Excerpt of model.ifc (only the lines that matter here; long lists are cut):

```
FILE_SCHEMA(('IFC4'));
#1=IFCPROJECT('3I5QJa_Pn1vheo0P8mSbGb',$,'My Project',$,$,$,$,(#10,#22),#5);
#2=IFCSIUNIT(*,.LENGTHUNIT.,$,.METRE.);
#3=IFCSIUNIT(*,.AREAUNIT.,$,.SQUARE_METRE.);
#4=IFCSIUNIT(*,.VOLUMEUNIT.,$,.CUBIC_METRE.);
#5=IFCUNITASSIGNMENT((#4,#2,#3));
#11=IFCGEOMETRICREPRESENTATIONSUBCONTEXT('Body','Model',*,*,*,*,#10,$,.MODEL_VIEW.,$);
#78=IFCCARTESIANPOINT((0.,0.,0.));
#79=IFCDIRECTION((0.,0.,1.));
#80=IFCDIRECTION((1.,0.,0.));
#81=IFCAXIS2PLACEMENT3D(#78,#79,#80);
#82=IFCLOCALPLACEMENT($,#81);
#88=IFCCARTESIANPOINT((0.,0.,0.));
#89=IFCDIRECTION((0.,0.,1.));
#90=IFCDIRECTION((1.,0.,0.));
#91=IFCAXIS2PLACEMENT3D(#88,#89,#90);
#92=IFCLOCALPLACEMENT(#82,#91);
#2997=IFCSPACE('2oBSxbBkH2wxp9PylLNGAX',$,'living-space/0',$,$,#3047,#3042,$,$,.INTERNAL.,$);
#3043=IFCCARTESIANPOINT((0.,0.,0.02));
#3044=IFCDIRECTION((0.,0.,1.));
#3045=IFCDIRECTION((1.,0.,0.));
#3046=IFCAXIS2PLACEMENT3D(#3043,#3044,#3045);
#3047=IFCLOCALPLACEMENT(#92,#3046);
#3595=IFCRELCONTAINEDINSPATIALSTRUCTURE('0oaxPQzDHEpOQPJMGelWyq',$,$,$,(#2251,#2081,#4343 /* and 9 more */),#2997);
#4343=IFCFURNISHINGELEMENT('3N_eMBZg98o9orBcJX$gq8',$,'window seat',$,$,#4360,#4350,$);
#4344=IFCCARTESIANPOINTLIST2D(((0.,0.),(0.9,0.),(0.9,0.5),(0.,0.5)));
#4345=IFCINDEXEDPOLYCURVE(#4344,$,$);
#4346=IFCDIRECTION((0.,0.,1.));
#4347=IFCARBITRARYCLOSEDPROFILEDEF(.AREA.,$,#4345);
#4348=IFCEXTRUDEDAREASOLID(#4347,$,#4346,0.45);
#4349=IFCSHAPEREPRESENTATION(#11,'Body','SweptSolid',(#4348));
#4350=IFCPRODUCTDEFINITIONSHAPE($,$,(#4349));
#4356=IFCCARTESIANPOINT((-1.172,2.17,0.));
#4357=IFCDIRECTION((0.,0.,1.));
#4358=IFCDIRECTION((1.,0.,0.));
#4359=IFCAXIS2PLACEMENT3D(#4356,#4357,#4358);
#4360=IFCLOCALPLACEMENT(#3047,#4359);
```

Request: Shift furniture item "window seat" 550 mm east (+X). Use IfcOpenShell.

```python
import ifcopenshell
import ifcopenshell.api.geometry
import ifcopenshell.util.placement
import ifcopenshell.util.unit

model = ifcopenshell.open("model.ifc")
unit_scale = ifcopenshell.util.unit.calculate_unit_scale(model)

item = model.by_guid("3N_eMBZg98o9orBcJX$gq8")
matrix = ifcopenshell.util.placement.get_local_placement(item.ObjectPlacement)
matrix[0, 3] += 0.55 / unit_scale
ifcopenshell.api.geometry.edit_object_placement(model, product=item, matrix=matrix, is_si=False)

print(ifcopenshell.util.placement.get_local_placement(item.ObjectPlacement).round(3) + 0.0)

model.write("model_edited.ifc")
```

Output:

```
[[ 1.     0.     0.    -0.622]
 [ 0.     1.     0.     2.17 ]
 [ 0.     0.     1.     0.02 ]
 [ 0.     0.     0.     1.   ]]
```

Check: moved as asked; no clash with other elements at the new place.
